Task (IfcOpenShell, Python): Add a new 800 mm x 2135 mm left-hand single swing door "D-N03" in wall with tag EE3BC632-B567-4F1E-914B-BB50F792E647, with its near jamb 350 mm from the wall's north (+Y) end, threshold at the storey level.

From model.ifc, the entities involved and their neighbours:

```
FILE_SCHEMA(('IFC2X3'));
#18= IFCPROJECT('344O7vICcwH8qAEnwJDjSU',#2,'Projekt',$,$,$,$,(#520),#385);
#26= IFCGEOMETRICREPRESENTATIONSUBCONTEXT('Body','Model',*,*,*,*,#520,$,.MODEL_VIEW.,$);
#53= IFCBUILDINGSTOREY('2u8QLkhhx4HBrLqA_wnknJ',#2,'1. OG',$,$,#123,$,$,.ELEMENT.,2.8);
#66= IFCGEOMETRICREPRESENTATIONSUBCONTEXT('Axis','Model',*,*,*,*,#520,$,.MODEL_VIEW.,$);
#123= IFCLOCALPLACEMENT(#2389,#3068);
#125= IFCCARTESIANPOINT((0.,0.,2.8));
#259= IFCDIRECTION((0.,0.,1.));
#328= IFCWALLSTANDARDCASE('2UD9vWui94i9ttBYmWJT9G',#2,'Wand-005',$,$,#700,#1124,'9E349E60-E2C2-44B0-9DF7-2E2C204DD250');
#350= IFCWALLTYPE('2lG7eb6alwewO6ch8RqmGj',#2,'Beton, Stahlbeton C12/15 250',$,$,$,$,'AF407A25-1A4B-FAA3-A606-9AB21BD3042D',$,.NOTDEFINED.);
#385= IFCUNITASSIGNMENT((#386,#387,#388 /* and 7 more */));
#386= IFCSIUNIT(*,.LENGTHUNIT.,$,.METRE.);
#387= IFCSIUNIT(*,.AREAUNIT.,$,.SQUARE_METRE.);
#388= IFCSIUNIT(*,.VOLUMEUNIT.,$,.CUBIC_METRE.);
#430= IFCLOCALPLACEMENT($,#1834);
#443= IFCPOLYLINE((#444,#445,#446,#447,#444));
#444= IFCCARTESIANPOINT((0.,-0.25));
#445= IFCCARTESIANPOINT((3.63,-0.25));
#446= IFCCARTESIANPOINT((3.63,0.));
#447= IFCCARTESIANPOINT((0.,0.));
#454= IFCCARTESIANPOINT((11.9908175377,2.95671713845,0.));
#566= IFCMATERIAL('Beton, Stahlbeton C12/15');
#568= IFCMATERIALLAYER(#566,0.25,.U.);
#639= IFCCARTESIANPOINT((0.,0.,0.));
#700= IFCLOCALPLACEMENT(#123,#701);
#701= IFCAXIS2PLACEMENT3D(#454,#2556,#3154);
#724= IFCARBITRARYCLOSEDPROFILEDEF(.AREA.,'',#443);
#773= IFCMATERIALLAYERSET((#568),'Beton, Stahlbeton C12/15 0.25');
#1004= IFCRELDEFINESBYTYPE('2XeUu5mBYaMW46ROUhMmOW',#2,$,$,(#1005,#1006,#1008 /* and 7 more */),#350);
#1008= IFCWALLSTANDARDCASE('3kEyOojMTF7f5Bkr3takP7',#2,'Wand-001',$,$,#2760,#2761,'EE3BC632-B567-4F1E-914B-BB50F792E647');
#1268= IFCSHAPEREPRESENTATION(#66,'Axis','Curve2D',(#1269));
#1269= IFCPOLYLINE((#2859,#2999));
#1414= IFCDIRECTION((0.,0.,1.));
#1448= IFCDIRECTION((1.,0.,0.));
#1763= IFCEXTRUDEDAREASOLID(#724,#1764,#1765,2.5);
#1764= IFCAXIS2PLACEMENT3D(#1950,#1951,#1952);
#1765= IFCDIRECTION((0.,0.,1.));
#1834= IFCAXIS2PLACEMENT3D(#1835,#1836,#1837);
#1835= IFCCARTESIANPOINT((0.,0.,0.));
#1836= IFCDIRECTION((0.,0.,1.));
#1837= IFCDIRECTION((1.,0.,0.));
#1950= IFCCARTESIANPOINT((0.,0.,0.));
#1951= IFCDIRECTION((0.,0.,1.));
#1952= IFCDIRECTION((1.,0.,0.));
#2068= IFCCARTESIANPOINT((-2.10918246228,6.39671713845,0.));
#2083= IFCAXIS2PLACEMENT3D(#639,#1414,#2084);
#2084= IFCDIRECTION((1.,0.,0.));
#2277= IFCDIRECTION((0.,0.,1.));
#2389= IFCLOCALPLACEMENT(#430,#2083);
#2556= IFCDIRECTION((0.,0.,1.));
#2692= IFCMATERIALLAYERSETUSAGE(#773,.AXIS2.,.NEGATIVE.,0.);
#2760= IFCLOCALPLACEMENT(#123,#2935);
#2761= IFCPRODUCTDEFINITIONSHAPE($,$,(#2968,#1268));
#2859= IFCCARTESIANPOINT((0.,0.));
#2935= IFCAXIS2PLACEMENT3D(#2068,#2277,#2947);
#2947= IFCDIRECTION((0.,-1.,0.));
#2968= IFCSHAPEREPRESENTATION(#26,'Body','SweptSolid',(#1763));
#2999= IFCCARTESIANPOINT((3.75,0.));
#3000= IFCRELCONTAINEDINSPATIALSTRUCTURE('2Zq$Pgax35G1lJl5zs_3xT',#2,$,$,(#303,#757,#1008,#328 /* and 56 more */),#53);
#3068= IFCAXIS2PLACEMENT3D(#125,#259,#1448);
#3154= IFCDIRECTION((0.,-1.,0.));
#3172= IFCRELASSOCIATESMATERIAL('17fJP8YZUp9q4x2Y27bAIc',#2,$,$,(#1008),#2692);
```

```python
import numpy as np
import ifcopenshell
import ifcopenshell.api.feature
import ifcopenshell.api.geometry
import ifcopenshell.api.root
import ifcopenshell.api.spatial
import ifcopenshell.api.type
import ifcopenshell.geom
import ifcopenshell.util.element
import ifcopenshell.util.placement
import ifcopenshell.util.representation
import ifcopenshell.util.shape
import ifcopenshell.util.unit

model = ifcopenshell.open("model.ifc")
unit_scale = ifcopenshell.util.unit.calculate_unit_scale(model)
settings = ifcopenshell.geom.settings()


def volume(element):
    """Net volume in cubic metres, openings subtracted."""
    shape = ifcopenshell.geom.create_shape(settings, element)
    return ifcopenshell.util.shape.get_volume(shape.geometry)


wall = model.by_id(1008)
storey = ifcopenshell.util.element.get_container(wall, ifc_class="IfcBuildingStorey")
context = ifcopenshell.util.representation.get_context(model, "Model", "Body", "MODEL_VIEW")
before = volume(wall)

width, height, from_end, sill = 0.8, 2.135, 0.35, 0.0  # metres

# The wall runs along its own X axis, and the end named is its -X end.
wall_shape = ifcopenshell.geom.create_shape(settings, wall)
x, y, z = ifcopenshell.util.shape.get_vertices(wall_shape.geometry).T
start = x.min() + from_end
face, thickness = float(y.min()), float(y.max() - y.min())
wall_matrix = ifcopenshell.util.placement.get_local_placement(wall.ObjectPlacement)
level = ifcopenshell.util.placement.get_local_placement(storey.ObjectPlacement)[2, 3]


def in_wall(x, y):
    """Placement at x, y metres in the wall's axes, at sill height."""
    matrix = wall_matrix.copy()
    matrix[:, 3] = wall_matrix @ np.array([x / unit_scale, y / unit_scale, 0.0, 1.0])
    matrix[2, 3] = level + sill / unit_scale
    return matrix


# Opening: a box that overshoots both wall faces by 50 mm.
opening = ifcopenshell.api.root.create_entity(model, ifc_class="IfcOpeningElement")
box = ifcopenshell.api.geometry.add_wall_representation(
    model, context=context, length=width, height=height, thickness=thickness + 0.1
)
ifcopenshell.api.geometry.assign_representation(model, product=opening, representation=box)
ifcopenshell.api.geometry.edit_object_placement(model, product=opening, matrix=in_wall(start, face - 0.05), is_si=False)
ifcopenshell.api.feature.add_feature(model, feature=opening, element=wall)

door = ifcopenshell.api.root.create_entity(model, ifc_class="IfcDoor", name="D-N03")
door.OverallWidth, door.OverallHeight = width / unit_scale, height / unit_scale
body = ifcopenshell.api.geometry.add_door_representation(
    model,
    context=context,
    overall_width=door.OverallWidth,
    overall_height=door.OverallHeight,
    operation_type="SINGLE_SWING_LEFT",
    lining_properties={"LiningDepth": thickness / unit_scale, "ThresholdDepth": thickness / unit_scale},
)
ifcopenshell.api.geometry.assign_representation(model, product=door, representation=body)
ifcopenshell.api.spatial.assign_container(model, products=[door], relating_structure=storey)
fills = ifcopenshell.api.feature.add_filling(model, opening=opening, element=door)
fills.OwnerHistory = door.OwnerHistory  # required in IFC2X3

# IFC2X3 keeps the operation on the door style.
style = ifcopenshell.api.root.create_entity(model, ifc_class="IfcDoorStyle", name="D-N03")
style.OperationType, style.ConstructionType = "SINGLE_SWING_LEFT", "NOTDEFINED"
style.ParameterTakesPrecedence = style.Sizeable = False
ifcopenshell.api.type.assign_type(model, related_objects=[door], relating_type=style)

# The lining spans the wall, so the door starts at the wall face.
ifcopenshell.api.geometry.edit_object_placement(model, product=door, matrix=in_wall(start, face), is_si=False)

after = volume(wall)

print(f"wall volume {before:.3f} -> {after:.3f} m3")

model.write("model_updated.ifc")
```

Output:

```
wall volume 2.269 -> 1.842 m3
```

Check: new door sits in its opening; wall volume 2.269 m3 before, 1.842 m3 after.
